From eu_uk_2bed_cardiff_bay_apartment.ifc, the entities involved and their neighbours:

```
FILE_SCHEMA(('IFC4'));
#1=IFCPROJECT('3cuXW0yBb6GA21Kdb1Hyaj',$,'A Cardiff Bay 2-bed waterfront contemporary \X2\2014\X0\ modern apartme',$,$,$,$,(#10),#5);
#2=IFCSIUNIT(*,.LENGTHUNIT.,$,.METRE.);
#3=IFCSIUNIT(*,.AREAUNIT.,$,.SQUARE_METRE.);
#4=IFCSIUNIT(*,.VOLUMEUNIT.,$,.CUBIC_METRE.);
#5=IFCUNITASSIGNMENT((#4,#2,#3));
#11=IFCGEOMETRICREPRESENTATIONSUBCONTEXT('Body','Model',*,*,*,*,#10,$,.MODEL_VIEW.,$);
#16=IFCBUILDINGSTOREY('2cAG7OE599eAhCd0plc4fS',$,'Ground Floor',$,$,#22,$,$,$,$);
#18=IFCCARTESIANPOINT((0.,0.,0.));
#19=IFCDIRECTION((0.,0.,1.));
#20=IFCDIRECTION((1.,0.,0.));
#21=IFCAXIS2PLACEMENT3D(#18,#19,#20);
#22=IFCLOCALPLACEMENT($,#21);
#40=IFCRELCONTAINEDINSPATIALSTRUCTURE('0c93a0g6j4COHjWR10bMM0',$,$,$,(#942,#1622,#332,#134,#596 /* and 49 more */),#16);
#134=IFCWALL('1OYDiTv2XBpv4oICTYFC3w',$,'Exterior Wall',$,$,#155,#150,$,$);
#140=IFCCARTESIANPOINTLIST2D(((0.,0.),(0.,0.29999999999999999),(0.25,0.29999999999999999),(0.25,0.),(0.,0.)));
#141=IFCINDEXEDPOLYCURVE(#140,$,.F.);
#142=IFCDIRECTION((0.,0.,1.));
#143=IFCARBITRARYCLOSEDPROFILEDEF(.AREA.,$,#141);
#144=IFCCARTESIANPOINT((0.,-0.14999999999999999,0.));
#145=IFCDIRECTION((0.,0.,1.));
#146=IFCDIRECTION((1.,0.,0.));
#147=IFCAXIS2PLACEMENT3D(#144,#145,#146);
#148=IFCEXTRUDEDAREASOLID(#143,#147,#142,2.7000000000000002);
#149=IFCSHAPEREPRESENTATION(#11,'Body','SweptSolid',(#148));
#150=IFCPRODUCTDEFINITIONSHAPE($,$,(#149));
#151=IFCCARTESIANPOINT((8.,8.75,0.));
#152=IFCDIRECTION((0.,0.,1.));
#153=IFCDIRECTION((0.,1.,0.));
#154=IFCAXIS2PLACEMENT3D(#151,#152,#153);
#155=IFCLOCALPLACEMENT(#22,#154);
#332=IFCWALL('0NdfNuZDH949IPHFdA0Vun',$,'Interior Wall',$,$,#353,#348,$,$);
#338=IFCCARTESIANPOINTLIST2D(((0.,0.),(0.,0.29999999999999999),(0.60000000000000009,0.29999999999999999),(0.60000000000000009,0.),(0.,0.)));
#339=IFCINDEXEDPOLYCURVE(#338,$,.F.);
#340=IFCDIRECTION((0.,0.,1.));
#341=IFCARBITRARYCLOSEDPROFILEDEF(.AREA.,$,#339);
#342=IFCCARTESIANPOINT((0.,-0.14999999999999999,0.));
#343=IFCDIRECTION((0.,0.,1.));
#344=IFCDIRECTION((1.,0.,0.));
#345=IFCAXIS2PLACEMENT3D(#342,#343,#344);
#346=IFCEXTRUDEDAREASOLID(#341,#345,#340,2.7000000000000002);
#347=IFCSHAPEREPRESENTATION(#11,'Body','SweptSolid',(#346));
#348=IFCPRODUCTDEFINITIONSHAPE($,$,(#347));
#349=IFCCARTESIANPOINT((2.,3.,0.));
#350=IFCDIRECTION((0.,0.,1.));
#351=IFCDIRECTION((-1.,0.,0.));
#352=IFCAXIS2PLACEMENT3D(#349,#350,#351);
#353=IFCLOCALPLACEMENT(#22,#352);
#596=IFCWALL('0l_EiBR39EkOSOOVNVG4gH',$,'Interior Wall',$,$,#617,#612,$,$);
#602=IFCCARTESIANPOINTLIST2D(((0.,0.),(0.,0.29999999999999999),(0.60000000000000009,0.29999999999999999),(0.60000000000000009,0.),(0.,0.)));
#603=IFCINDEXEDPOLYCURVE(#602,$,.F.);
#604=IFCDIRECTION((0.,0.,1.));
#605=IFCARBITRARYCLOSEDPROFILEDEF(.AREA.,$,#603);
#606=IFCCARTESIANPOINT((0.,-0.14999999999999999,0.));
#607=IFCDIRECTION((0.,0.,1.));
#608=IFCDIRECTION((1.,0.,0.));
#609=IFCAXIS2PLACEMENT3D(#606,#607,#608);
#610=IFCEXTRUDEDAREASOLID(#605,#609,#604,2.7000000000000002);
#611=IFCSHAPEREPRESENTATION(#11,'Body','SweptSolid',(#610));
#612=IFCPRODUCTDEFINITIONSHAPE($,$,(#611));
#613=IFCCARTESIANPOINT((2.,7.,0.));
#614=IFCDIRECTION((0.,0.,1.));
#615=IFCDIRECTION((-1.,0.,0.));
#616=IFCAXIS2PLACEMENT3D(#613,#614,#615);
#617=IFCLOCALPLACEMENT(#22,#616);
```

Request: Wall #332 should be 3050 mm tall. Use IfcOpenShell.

```python
import ifcopenshell
import ifcopenshell.geom
import ifcopenshell.util.representation
import ifcopenshell.util.shape

model = ifcopenshell.open("eu_uk_2bed_cardiff_bay_apartment.ifc")
settings = ifcopenshell.geom.settings()


def volume(element):
    """Net volume in cubic metres, openings subtracted."""
    shape = ifcopenshell.geom.create_shape(settings, element)
    return ifcopenshell.util.shape.get_volume(shape.geometry)


wall = model.by_guid("0NdfNuZDH949IPHFdA0Vun")
before = volume(wall)

body = ifcopenshell.util.representation.get_representation(wall, "Model", "Body")
solid = body.Items[0]
old_height = solid.Depth
solid.Depth = 3.05
after = volume(wall)

print(f"height {old_height:g} -> {solid.Depth:g}, volume {before:.3f} -> {after:.3f} m3")

model.write("eu_uk_2bed_cardiff_bay_apartment_updated.ifc")
```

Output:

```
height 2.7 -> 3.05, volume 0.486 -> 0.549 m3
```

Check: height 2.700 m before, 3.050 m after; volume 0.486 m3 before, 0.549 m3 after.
